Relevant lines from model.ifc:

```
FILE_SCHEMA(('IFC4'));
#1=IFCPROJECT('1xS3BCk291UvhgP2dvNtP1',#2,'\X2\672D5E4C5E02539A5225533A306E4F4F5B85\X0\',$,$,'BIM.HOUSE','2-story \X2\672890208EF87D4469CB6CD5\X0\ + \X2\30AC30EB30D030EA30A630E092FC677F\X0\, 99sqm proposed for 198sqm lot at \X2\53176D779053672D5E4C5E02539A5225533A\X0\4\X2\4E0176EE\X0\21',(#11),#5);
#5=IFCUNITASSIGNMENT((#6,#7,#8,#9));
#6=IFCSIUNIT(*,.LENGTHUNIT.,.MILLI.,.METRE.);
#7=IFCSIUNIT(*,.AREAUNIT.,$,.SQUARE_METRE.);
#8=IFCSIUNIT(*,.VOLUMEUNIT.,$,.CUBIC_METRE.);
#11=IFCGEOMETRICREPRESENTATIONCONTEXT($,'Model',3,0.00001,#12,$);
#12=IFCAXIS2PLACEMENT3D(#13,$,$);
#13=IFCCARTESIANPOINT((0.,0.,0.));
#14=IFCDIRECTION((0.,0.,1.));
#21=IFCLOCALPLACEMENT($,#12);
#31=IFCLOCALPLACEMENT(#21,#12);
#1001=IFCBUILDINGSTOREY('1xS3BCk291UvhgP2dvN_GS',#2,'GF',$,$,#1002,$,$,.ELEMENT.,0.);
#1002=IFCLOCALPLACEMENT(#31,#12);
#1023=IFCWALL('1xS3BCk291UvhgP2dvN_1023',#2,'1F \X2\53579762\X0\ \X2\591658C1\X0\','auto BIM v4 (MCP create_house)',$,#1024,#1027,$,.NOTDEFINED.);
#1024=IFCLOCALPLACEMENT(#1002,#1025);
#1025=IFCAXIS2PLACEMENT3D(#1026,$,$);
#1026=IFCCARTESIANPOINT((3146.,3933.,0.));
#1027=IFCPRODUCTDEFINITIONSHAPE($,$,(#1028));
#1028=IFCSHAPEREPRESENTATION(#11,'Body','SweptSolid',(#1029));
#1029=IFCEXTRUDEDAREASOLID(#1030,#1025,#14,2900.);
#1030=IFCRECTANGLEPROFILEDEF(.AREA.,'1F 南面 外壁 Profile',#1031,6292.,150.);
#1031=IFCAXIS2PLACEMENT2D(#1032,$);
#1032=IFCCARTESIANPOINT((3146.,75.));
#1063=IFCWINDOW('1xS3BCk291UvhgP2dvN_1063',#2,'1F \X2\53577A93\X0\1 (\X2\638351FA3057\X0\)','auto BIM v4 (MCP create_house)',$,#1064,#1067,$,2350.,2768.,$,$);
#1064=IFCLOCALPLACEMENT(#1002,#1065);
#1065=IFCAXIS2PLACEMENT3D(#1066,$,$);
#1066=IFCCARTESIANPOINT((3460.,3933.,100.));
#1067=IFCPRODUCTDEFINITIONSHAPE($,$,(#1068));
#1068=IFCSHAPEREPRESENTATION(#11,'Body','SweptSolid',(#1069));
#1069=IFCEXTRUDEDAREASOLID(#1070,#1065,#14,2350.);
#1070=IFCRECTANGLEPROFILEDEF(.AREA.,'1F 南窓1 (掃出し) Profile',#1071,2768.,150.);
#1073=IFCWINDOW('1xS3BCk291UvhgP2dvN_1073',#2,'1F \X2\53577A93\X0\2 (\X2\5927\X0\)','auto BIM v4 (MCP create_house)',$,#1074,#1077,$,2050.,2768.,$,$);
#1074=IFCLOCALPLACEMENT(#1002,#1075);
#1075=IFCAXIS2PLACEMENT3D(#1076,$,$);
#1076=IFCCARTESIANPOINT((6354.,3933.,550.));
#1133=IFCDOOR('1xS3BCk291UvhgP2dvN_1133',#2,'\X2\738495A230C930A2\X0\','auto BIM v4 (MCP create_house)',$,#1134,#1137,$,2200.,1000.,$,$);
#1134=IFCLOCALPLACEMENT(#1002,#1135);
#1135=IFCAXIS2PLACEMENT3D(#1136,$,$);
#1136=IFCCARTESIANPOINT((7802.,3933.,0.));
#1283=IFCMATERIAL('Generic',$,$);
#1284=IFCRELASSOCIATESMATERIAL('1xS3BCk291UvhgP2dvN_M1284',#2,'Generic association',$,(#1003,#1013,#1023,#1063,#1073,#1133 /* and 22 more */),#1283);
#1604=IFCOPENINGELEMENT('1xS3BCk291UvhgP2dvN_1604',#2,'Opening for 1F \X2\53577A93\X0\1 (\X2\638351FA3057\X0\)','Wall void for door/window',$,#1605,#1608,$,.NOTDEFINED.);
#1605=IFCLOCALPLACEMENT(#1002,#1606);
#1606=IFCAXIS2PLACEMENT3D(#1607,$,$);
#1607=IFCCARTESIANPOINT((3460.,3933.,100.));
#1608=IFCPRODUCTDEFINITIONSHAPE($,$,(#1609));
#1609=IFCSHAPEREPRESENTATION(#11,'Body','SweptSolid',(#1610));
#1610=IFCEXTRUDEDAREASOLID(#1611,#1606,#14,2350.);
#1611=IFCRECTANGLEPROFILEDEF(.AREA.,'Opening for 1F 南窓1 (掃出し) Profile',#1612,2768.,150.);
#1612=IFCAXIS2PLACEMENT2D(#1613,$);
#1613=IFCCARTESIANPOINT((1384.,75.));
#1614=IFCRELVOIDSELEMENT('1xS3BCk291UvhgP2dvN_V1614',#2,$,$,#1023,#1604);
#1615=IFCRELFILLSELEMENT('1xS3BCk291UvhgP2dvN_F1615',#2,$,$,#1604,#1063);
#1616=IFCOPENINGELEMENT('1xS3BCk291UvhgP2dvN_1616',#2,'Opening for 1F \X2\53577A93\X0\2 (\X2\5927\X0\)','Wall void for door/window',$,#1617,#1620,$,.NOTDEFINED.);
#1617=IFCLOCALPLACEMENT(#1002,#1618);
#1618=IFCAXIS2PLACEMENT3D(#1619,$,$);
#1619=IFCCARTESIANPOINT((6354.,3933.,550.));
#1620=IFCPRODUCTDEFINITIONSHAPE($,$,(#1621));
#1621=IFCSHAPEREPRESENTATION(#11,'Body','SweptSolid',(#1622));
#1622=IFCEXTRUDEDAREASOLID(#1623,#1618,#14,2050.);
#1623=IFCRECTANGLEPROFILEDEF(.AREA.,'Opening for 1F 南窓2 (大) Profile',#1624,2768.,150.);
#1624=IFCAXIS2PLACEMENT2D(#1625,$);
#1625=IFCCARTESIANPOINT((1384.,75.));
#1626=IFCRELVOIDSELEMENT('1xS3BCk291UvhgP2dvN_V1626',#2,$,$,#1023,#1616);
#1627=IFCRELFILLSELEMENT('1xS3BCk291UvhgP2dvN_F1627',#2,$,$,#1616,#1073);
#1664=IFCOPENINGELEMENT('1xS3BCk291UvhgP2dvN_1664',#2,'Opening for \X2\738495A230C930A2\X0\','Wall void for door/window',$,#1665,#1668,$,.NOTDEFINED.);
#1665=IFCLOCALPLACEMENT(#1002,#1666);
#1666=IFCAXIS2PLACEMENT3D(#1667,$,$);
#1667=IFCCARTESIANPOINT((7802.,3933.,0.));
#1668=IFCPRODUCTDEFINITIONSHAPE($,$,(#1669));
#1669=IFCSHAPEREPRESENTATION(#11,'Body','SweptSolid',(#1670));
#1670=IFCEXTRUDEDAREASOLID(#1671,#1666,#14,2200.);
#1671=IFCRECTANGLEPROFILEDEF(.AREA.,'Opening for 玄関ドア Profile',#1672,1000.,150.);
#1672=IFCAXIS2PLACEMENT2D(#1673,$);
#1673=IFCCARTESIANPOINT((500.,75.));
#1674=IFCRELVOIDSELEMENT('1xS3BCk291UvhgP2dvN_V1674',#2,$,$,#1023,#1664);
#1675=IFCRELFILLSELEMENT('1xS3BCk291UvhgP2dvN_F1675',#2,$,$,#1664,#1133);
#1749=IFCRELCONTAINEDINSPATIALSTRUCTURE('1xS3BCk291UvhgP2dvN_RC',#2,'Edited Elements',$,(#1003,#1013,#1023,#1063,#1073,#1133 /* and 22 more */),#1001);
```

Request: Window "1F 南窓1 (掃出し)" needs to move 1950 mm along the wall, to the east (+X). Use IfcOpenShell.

```python
import ifcopenshell
import ifcopenshell.api.geometry
import ifcopenshell.util.placement

model = ifcopenshell.open("model.ifc")

window = model.by_guid("1xS3BCk291UvhgP2dvN_1063")
opening = window.FillsVoids[0].RelatingOpeningElement
wall = opening.VoidsElements[0].RelatingBuildingElement

wall_matrix = ifcopenshell.util.placement.get_local_placement(wall.ObjectPlacement)
shift = wall_matrix[:3, 0] * 1950.0
before = ifcopenshell.util.placement.get_local_placement(window.ObjectPlacement)[:3, 3].copy()

# The window is not placed relative to its opening, so move both.
for product in (opening, window):
    matrix = ifcopenshell.util.placement.get_local_placement(product.ObjectPlacement)
    matrix[:3, 3] += shift
    ifcopenshell.api.geometry.edit_object_placement(model, product=product, matrix=matrix, is_si=False)

after = ifcopenshell.util.placement.get_local_placement(window.ObjectPlacement)[:3, 3]
print("window moved by", (after - before).round(3) + 0.0)

model.write("model_v2.ifc")
```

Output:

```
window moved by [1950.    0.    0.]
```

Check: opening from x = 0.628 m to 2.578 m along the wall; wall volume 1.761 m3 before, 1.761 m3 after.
